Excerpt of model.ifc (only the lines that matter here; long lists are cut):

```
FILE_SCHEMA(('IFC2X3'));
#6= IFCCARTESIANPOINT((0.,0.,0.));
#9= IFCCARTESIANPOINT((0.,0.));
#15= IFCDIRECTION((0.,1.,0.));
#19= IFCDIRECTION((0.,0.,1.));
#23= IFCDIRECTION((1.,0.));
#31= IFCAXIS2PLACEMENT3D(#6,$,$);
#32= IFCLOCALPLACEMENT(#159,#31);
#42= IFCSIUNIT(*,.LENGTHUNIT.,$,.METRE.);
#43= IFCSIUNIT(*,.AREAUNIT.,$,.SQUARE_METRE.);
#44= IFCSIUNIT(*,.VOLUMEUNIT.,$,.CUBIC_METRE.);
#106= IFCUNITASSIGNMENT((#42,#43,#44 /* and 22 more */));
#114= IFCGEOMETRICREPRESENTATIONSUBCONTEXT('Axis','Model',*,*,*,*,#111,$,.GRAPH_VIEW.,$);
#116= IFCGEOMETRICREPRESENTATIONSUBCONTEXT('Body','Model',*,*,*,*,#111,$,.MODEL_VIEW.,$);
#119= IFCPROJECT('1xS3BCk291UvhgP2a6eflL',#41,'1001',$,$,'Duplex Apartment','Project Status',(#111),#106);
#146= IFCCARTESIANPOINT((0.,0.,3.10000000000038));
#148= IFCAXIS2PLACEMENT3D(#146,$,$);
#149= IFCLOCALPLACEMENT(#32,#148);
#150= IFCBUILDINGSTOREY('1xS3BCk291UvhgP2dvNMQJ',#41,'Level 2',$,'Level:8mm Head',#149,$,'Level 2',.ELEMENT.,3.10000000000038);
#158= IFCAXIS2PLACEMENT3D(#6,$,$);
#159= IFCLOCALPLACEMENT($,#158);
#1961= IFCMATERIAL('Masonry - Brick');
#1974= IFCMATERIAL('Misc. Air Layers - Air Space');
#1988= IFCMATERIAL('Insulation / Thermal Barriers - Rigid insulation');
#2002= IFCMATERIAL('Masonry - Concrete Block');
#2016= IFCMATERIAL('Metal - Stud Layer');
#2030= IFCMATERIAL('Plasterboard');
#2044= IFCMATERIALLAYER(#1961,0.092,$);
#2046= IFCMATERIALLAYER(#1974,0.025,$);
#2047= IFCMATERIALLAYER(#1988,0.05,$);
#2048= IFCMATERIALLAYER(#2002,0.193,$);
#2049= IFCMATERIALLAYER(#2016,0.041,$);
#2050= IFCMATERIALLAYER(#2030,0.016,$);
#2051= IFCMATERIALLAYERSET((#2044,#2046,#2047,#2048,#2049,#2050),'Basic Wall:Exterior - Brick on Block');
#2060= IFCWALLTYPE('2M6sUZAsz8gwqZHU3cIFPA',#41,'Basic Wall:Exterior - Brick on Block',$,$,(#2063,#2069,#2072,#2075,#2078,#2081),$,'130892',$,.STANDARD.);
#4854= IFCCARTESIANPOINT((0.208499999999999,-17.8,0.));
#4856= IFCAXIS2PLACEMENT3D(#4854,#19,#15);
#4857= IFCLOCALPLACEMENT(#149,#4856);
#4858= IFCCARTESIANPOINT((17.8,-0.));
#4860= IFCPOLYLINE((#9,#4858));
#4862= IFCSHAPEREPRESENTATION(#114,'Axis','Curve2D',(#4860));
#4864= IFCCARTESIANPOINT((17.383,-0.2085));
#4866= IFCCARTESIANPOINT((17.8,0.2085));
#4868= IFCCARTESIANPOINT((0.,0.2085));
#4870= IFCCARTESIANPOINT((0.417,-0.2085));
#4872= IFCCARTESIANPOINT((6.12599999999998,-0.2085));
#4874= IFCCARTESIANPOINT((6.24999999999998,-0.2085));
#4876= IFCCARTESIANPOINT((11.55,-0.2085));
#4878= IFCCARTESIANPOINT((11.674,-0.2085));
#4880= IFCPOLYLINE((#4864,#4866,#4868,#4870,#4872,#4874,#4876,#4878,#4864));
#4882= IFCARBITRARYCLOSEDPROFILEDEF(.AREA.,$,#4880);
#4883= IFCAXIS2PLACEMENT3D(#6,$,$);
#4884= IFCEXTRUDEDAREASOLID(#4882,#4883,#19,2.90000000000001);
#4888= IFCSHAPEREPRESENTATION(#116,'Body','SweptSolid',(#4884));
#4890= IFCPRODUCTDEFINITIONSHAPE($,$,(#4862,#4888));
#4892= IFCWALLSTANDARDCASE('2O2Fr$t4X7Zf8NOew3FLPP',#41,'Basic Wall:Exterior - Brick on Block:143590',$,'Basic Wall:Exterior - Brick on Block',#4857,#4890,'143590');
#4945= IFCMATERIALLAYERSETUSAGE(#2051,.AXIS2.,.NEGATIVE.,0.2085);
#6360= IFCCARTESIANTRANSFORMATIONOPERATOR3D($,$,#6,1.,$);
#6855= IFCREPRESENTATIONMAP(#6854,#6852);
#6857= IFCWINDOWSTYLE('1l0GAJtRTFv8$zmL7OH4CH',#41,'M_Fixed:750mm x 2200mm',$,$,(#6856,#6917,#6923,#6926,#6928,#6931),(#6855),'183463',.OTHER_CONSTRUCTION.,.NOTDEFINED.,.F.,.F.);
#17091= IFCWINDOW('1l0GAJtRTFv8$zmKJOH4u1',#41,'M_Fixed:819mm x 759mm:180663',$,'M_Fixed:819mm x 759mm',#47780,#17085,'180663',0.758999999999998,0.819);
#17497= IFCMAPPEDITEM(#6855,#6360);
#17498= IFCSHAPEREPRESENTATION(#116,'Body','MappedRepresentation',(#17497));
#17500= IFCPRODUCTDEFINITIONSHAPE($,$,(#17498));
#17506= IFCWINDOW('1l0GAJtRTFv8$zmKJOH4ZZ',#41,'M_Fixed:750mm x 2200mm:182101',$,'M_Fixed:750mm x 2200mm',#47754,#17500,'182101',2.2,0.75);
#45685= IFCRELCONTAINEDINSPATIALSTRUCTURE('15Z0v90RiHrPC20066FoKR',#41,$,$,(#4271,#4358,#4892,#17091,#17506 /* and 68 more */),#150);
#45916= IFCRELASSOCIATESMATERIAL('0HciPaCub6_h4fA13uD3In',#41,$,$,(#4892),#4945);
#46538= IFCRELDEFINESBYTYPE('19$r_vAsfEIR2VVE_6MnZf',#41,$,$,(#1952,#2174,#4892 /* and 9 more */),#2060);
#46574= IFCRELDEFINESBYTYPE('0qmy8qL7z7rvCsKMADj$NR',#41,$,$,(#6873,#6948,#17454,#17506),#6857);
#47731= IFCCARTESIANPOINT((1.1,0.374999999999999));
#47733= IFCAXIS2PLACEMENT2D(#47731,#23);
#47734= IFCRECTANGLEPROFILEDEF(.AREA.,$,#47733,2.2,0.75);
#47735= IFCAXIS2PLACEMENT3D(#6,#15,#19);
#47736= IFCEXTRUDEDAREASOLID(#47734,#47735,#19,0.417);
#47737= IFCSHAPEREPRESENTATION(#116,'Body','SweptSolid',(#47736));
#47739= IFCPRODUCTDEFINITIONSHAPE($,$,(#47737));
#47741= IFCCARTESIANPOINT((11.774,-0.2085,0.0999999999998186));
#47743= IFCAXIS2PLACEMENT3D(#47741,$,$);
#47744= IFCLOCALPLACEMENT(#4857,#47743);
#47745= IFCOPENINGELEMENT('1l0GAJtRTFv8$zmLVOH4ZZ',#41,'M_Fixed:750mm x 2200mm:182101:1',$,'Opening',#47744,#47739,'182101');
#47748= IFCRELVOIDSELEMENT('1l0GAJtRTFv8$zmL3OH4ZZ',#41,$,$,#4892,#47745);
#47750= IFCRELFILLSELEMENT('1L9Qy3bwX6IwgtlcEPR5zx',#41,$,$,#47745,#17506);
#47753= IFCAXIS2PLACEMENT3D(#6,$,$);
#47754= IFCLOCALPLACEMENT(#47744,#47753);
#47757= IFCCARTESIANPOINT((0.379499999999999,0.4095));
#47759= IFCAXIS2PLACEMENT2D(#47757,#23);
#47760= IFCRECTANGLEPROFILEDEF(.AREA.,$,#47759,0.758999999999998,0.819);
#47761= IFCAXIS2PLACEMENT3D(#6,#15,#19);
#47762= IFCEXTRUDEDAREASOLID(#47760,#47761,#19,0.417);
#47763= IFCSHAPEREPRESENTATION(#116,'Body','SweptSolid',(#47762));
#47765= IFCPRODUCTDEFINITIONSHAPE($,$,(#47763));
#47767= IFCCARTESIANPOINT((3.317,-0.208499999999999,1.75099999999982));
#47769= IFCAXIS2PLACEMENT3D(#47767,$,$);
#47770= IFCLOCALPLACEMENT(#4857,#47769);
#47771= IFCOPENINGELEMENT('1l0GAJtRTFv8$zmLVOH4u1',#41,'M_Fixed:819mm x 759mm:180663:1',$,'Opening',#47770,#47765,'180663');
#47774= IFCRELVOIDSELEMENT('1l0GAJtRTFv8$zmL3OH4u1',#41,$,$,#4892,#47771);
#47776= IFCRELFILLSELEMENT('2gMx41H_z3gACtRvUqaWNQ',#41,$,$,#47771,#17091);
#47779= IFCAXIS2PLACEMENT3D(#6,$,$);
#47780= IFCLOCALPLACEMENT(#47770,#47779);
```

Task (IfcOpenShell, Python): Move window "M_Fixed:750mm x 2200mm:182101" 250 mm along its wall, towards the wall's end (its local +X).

```python
import ifcopenshell
import ifcopenshell.api.geometry
import ifcopenshell.util.placement
import ifcopenshell.util.unit

model = ifcopenshell.open("model.ifc")
unit_scale = ifcopenshell.util.unit.calculate_unit_scale(model)

window = model.by_guid("1l0GAJtRTFv8$zmKJOH4ZZ")
opening = window.FillsVoids[0].RelatingOpeningElement
wall = opening.VoidsElements[0].RelatingBuildingElement

wall_matrix = ifcopenshell.util.placement.get_local_placement(wall.ObjectPlacement)
shift = wall_matrix[:3, 0] * 0.25 / unit_scale
before = ifcopenshell.util.placement.get_local_placement(window.ObjectPlacement)[:3, 3].copy()

# The window is placed relative to its opening, so it follows when the opening moves.
matrix = ifcopenshell.util.placement.get_local_placement(opening.ObjectPlacement)
matrix[:3, 3] += shift
ifcopenshell.api.geometry.edit_object_placement(
    model, product=opening, matrix=matrix, is_si=False, should_transform_children=True
)

after = ifcopenshell.util.placement.get_local_placement(window.ObjectPlacement)[:3, 3]
print("window moved by", (after - before).round(3) + 0.0)

model.write("model_updated.ifc")
```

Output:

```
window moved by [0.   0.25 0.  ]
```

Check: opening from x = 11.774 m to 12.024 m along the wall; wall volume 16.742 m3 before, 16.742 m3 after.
